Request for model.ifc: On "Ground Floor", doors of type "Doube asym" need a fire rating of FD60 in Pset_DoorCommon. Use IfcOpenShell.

First a look at what the model holds.

```python
import ifcopenshell
import ifcopenshell.util.element

model = ifcopenshell.open("model.ifc")
print(model.schema)
storey = next(s for s in model.by_type("IfcBuildingStorey") if s.Name == "Ground Floor")
doors = [e for e in ifcopenshell.util.element.get_decomposition(storey) if e.is_a("IfcDoor")]
seen = {}
for e in doors:
    element_type = ifcopenshell.util.element.get_type(e)
    key = (element_type.Name if element_type != e and element_type else None, ifcopenshell.util.element.get_pset(e, "Pset_DoorCommon", "FireRating"))
    seen[key] = seen.get(key, 0) + 1
for (name, value), count in sorted(seen.items(), key=str):
    print(count, "x", name, "|", value)
```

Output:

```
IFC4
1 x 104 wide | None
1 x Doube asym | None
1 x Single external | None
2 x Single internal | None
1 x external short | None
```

```python
import ifcopenshell
import ifcopenshell.api.pset
import ifcopenshell.util.element

model = ifcopenshell.open("model.ifc")

storey = next(s for s in model.by_type("IfcBuildingStorey") if s.Name == "Ground Floor")
doors = [e for e in ifcopenshell.util.element.get_decomposition(storey) if e.is_a("IfcDoor")]

count = 0
for e in doors:
    element_type = ifcopenshell.util.element.get_type(e)
    if element_type in (None, e) or element_type.Name != "Doube asym":
        continue
    # add_pset returns the element's existing set when there is one.
    pset = ifcopenshell.api.pset.add_pset(model, product=e, name="Pset_DoorCommon")
    ifcopenshell.api.pset.edit_pset(model, pset=pset, properties={"FireRating": "FD60"})
    count += 1

print(count, "doors updated")

model.write("model_edited.ifc")
```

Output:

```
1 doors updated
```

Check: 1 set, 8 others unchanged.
